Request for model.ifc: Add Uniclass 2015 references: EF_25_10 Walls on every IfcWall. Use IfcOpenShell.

First a look at what the model holds.

```python
import ifcopenshell

model = ifcopenshell.open("model.ifc")
print(model.schema)
print("classifications:", [c.Name for c in model.by_type("IfcClassification")])
for ifc_class in ("IfcDoor", "IfcRoof", "IfcStair", "IfcWall", "IfcWindow"):
    print(ifc_class, len(model.by_type(ifc_class)))
```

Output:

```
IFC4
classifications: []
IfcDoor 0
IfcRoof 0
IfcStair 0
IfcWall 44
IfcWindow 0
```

```python
import ifcopenshell
import ifcopenshell.api.classification

model = ifcopenshell.open("model.ifc")

system = ifcopenshell.api.classification.add_classification(model, classification="Uniclass 2015")

codes = {
    "IfcWall": ("EF_25_10", "Walls"),
}
for ifc_class, (code, name) in codes.items():
    products = model.by_type(ifc_class)
    ifcopenshell.api.classification.add_reference(
        model, products=products, classification=system, identification=code, name=name
    )
    print(code, len(products))

model.write("model_v2.ifc")
```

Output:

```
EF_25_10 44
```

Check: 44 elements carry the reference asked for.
